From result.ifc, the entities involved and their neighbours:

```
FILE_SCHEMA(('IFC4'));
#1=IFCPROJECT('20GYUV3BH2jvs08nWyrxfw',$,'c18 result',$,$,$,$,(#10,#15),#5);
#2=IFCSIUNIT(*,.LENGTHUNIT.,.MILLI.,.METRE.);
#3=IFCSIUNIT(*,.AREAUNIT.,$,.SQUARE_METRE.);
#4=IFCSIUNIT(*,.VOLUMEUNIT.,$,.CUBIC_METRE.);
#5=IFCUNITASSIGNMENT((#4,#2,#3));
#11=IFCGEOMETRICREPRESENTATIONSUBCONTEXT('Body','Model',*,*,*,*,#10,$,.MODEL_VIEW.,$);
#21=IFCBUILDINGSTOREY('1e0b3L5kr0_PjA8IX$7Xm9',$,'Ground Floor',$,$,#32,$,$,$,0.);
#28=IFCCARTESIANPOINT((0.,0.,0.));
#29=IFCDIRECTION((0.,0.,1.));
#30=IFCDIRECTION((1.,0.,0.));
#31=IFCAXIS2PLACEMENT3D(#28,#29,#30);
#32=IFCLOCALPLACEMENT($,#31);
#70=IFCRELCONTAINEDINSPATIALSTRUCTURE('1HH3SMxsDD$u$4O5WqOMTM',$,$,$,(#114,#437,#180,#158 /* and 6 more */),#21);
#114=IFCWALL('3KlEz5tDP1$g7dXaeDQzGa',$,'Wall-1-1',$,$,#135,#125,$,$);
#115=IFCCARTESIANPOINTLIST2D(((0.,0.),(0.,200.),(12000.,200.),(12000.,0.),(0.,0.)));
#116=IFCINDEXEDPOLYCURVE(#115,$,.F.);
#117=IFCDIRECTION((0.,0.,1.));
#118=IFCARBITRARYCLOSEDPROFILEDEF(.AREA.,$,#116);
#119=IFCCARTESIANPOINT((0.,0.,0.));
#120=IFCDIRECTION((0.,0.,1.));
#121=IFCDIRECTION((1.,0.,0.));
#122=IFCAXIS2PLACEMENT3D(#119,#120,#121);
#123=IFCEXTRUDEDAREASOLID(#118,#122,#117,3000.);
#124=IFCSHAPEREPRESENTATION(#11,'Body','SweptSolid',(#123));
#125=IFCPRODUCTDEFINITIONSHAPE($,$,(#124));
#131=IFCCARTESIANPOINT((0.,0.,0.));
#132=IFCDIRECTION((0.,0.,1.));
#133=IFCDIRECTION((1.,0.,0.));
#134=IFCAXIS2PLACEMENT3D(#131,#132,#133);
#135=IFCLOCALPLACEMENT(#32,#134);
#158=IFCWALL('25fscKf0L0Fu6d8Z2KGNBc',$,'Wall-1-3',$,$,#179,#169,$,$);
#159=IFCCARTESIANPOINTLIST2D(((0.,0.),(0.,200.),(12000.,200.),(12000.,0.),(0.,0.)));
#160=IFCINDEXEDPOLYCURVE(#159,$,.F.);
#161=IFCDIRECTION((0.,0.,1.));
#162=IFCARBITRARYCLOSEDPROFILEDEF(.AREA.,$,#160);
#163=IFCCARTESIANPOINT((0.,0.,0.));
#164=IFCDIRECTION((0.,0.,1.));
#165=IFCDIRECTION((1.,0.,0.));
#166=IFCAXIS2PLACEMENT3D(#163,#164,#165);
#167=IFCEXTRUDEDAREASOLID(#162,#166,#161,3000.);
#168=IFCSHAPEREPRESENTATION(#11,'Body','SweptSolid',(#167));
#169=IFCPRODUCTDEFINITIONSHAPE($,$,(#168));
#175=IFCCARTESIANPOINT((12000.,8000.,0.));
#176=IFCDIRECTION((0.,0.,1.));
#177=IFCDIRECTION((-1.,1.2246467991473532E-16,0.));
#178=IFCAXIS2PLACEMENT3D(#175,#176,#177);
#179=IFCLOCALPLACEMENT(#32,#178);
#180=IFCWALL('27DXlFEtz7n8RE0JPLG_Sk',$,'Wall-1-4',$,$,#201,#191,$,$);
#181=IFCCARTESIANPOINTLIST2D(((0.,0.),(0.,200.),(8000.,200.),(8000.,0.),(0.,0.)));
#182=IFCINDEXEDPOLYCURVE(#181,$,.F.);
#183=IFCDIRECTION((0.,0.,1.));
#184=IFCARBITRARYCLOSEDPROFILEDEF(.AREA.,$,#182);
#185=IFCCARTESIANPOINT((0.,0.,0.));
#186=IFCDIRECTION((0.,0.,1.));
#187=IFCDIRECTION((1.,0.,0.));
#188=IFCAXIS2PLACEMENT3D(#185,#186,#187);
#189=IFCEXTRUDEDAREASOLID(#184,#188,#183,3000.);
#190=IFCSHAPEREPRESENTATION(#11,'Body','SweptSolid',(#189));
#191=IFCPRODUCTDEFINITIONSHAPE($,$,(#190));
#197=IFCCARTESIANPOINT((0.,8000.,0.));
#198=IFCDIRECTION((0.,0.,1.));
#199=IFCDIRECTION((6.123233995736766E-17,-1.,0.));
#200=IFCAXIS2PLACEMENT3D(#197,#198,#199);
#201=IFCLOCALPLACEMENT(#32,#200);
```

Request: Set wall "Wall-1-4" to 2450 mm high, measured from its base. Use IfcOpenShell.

```python
import ifcopenshell
import ifcopenshell.geom
import ifcopenshell.util.representation
import ifcopenshell.util.shape

model = ifcopenshell.open("result.ifc")
settings = ifcopenshell.geom.settings()


def volume(element):
    """Net volume in cubic metres, openings subtracted."""
    shape = ifcopenshell.geom.create_shape(settings, element)
    return ifcopenshell.util.shape.get_volume(shape.geometry)


wall = model.by_guid("27DXlFEtz7n8RE0JPLG_Sk")
before = volume(wall)

body = ifcopenshell.util.representation.get_representation(wall, "Model", "Body")
solid = body.Items[0]
old_height = solid.Depth
solid.Depth = 2450.0
after = volume(wall)

print(f"height {old_height:g} -> {solid.Depth:g}, volume {before:.3f} -> {after:.3f} m3")

model.write("result_updated.ifc")
```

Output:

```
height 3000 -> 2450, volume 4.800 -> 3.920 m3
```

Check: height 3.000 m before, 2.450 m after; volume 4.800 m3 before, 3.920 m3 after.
